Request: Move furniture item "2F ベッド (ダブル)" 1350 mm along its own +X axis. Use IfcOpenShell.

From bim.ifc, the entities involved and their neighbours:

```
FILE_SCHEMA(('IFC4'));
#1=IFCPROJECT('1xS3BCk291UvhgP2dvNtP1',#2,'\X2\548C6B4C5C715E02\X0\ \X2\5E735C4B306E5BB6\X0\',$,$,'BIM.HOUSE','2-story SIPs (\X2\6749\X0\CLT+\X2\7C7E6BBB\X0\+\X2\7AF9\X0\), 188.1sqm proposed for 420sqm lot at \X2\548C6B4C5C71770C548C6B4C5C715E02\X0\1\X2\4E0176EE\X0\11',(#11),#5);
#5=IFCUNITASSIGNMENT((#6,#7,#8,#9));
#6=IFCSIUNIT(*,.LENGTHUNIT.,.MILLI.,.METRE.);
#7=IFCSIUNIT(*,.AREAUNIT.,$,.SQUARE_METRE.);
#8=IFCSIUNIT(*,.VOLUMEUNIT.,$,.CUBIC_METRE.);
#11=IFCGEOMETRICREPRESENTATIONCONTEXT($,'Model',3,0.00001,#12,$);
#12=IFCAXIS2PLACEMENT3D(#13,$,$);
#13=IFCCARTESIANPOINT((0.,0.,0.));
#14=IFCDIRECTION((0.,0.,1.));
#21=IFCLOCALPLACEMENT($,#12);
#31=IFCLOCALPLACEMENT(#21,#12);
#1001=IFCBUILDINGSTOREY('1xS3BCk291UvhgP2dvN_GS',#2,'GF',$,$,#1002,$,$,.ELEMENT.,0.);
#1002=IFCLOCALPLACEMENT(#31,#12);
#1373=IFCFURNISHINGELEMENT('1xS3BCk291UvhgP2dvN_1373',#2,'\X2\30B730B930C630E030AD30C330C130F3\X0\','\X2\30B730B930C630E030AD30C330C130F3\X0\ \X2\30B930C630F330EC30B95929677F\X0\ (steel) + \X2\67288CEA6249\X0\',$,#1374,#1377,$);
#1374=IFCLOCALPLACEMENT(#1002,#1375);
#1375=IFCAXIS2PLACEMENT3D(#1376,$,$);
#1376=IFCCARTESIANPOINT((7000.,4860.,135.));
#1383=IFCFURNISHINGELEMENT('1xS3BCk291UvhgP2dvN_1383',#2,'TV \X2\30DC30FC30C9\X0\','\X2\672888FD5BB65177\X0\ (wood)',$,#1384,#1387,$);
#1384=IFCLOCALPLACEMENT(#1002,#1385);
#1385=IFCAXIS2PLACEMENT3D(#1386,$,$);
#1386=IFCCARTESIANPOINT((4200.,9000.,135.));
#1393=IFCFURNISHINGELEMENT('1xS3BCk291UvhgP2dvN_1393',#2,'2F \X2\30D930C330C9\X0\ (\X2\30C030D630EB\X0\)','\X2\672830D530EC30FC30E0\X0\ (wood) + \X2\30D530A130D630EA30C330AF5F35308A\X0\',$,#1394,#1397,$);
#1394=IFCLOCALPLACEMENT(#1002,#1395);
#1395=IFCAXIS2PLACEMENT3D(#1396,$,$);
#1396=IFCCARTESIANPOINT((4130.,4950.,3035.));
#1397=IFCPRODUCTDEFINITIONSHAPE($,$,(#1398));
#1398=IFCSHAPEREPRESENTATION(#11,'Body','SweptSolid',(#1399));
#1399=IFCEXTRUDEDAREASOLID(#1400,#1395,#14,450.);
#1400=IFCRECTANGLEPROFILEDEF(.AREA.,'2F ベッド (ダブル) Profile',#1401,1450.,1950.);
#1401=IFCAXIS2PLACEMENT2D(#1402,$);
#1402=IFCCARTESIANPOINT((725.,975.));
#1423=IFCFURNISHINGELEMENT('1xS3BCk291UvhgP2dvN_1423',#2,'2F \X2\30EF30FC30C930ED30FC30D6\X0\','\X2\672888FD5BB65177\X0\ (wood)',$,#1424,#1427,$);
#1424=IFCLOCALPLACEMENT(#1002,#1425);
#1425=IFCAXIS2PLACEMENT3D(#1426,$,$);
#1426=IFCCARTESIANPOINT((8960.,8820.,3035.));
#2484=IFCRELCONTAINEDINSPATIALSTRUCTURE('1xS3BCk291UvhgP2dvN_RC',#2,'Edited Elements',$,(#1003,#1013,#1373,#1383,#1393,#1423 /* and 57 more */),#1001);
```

```python
import ifcopenshell
import ifcopenshell.api.geometry
import ifcopenshell.util.placement

model = ifcopenshell.open("bim.ifc")

item = model.by_guid("1xS3BCk291UvhgP2dvN_1393")
matrix = ifcopenshell.util.placement.get_local_placement(item.ObjectPlacement)
matrix[:3, 3] += matrix[:3, 0] * 1350.0
ifcopenshell.api.geometry.edit_object_placement(model, product=item, matrix=matrix, is_si=False)

print(ifcopenshell.util.placement.get_local_placement(item.ObjectPlacement).round(3) + 0.0)

model.write("bim_rev.ifc")
```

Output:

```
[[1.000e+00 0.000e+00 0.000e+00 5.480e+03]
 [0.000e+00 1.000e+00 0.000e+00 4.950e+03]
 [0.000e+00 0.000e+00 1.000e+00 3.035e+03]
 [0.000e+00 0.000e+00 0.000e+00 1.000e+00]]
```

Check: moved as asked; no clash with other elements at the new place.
